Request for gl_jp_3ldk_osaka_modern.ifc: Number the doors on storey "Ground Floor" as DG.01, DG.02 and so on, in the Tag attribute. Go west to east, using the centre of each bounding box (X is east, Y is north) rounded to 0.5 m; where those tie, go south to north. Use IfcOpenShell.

First a look at what the model holds.

```python
import ifcopenshell
import ifcopenshell.util.element
import ifcopenshell.util.placement

model = ifcopenshell.open("gl_jp_3ldk_osaka_modern.ifc")
print(model.schema)
storey = next(s for s in model.by_type("IfcBuildingStorey") if s.Name == "Ground Floor")
doors = [e for e in ifcopenshell.util.element.get_decomposition(storey) if e.is_a("IfcDoor")]
for e in sorted(doors, key=lambda e: e.id()):
    origin = ifcopenshell.util.placement.get_local_placement(e.ObjectPlacement)[:3, 3]
    print(e.id(), e.Tag, e.Name, origin.round(2) + 0.0, sep=" | ")
```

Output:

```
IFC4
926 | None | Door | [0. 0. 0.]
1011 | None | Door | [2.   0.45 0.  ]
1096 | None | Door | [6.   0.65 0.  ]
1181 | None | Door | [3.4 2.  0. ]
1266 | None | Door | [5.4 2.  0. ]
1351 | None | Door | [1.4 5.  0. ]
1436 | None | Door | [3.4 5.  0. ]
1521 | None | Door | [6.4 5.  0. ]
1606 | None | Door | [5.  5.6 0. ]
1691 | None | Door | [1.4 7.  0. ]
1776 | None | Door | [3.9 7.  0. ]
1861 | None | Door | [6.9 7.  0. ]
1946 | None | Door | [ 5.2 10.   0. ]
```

```python
import ifcopenshell
import ifcopenshell.geom
import ifcopenshell.util.element
import ifcopenshell.util.shape

model = ifcopenshell.open("gl_jp_3ldk_osaka_modern.ifc")
settings = ifcopenshell.geom.settings()
settings.set("use-world-coords", True)


def centre(element):
    shape = ifcopenshell.geom.create_shape(settings, element)
    return ifcopenshell.util.shape.get_bbox_centroid(shape.geometry)


storey = next(s for s in model.by_type("IfcBuildingStorey") if s.Name == "Ground Floor")
doors = [e for e in ifcopenshell.util.element.get_decomposition(storey) if e.is_a("IfcDoor")]

# Insertion points can sit at a corner or the storey origin, so sort by the geometry (in metres).
centres = {e: centre(e) for e in doors}
doors.sort(key=lambda e: (round(centres[e][0] / 0.5), centres[e][1]))

for i, e in enumerate(doors, start=1):
    number = f"DG.{i:02d}"
    e.Tag = number
    print(e.id(), number)

model.write("gl_jp_3ldk_osaka_modern-out.ifc")
```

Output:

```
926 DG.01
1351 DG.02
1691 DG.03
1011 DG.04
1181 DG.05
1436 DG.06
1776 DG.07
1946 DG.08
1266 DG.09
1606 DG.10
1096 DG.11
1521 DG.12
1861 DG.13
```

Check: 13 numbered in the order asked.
